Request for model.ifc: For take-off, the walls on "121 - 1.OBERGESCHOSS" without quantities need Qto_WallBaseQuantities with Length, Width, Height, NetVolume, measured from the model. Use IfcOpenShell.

First a look at what the model holds.

```python
import ifcopenshell
import ifcopenshell.util.element
import ifcopenshell.util.unit

model = ifcopenshell.open("model.ifc")
print(model.schema)
for unit_type in ("LENGTHUNIT", "AREAUNIT", "VOLUMEUNIT"):
    print(unit_type, ifcopenshell.util.unit.calculate_unit_scale(model, unit_type))
storey = next(s for s in model.by_type("IfcBuildingStorey") if s.Name == "121 - 1.OBERGESCHOSS")
walls = [e for e in ifcopenshell.util.element.get_decomposition(storey) if e.is_a("IfcWall")]
for e in sorted(walls, key=lambda e: e.id()):
    print(e.id(), e.is_a(), e.Name, list(ifcopenshell.util.element.get_psets(e, qtos_only=True)), sep=" | ")
```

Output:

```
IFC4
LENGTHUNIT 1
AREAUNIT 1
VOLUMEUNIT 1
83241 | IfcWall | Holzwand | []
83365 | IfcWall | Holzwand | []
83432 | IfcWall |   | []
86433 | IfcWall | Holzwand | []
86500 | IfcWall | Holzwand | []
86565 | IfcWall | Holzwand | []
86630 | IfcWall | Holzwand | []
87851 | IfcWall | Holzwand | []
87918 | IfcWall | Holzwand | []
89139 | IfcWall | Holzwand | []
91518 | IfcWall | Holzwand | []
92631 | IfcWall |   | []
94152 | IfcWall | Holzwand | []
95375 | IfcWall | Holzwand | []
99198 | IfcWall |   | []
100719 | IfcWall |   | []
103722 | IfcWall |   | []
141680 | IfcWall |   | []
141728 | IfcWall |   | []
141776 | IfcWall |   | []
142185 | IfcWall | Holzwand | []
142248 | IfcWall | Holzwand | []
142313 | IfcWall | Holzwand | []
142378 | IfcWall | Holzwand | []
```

```python
import ifcopenshell
import ifcopenshell.api.pset
import ifcopenshell.geom
import ifcopenshell.util.element
import ifcopenshell.util.shape
import ifcopenshell.util.unit

model = ifcopenshell.open("model.ifc")
unit_scale = ifcopenshell.util.unit.calculate_unit_scale(model)
volume_scale = ifcopenshell.util.unit.calculate_unit_scale(model, "VOLUMEUNIT")
settings = ifcopenshell.geom.settings()

storey = next(s for s in model.by_type("IfcBuildingStorey") if s.Name == "121 - 1.OBERGESCHOSS")
walls = [e for e in ifcopenshell.util.element.get_decomposition(storey) if e.is_a("IfcWall")]

for e in sorted(walls, key=lambda e: e.id()):
    if ifcopenshell.util.element.get_psets(e, qtos_only=True, should_inherit=False):
        continue
    # Geometry comes back in metres, in the element's own axes.
    shape = ifcopenshell.geom.create_shape(settings, e)
    values = {
        "Length": ifcopenshell.util.shape.get_x(shape.geometry) / unit_scale,
        "Width": ifcopenshell.util.shape.get_y(shape.geometry) / unit_scale,
        "Height": ifcopenshell.util.shape.get_z(shape.geometry) / unit_scale,
        "NetVolume": ifcopenshell.util.shape.get_volume(shape.geometry) / volume_scale,
    }
    qto = ifcopenshell.api.pset.add_qto(model, product=e, name="Qto_WallBaseQuantities")
    ifcopenshell.api.pset.edit_qto(model, qto=qto, properties=values)
    print(e.id(), {k: round(v, 3) for k, v in values.items()})

model.write("model_rev.ifc")
```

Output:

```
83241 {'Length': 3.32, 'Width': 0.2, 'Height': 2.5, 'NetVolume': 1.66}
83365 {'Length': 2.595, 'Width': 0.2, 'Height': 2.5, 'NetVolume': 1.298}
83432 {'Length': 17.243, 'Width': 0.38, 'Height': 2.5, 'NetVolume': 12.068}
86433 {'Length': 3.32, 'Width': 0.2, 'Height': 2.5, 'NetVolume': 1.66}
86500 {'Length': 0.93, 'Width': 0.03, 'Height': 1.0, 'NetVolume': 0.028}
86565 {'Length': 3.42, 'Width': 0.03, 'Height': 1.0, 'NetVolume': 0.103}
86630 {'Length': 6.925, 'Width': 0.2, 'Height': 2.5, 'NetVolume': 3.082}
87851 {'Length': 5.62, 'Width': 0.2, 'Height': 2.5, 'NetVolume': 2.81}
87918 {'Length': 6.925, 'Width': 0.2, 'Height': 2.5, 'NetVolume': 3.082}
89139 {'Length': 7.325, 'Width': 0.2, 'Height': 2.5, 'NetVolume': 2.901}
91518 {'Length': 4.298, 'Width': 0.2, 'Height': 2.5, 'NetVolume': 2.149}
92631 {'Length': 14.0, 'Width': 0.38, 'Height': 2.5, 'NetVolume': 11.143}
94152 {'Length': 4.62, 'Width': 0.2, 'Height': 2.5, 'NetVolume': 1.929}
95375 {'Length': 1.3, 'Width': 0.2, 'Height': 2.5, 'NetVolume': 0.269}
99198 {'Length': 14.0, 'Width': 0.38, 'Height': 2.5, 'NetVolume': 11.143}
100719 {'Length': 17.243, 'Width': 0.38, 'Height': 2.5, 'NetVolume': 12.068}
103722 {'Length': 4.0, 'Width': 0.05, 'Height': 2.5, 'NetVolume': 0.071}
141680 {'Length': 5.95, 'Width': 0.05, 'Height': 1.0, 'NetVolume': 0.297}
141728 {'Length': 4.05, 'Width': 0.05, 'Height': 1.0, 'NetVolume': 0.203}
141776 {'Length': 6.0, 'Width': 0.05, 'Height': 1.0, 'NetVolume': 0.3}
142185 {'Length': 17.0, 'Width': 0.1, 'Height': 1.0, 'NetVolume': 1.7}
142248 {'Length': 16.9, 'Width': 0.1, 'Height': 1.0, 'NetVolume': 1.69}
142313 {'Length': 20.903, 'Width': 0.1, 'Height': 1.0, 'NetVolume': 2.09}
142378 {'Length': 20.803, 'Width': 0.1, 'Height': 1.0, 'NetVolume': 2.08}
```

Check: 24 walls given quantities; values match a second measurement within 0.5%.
